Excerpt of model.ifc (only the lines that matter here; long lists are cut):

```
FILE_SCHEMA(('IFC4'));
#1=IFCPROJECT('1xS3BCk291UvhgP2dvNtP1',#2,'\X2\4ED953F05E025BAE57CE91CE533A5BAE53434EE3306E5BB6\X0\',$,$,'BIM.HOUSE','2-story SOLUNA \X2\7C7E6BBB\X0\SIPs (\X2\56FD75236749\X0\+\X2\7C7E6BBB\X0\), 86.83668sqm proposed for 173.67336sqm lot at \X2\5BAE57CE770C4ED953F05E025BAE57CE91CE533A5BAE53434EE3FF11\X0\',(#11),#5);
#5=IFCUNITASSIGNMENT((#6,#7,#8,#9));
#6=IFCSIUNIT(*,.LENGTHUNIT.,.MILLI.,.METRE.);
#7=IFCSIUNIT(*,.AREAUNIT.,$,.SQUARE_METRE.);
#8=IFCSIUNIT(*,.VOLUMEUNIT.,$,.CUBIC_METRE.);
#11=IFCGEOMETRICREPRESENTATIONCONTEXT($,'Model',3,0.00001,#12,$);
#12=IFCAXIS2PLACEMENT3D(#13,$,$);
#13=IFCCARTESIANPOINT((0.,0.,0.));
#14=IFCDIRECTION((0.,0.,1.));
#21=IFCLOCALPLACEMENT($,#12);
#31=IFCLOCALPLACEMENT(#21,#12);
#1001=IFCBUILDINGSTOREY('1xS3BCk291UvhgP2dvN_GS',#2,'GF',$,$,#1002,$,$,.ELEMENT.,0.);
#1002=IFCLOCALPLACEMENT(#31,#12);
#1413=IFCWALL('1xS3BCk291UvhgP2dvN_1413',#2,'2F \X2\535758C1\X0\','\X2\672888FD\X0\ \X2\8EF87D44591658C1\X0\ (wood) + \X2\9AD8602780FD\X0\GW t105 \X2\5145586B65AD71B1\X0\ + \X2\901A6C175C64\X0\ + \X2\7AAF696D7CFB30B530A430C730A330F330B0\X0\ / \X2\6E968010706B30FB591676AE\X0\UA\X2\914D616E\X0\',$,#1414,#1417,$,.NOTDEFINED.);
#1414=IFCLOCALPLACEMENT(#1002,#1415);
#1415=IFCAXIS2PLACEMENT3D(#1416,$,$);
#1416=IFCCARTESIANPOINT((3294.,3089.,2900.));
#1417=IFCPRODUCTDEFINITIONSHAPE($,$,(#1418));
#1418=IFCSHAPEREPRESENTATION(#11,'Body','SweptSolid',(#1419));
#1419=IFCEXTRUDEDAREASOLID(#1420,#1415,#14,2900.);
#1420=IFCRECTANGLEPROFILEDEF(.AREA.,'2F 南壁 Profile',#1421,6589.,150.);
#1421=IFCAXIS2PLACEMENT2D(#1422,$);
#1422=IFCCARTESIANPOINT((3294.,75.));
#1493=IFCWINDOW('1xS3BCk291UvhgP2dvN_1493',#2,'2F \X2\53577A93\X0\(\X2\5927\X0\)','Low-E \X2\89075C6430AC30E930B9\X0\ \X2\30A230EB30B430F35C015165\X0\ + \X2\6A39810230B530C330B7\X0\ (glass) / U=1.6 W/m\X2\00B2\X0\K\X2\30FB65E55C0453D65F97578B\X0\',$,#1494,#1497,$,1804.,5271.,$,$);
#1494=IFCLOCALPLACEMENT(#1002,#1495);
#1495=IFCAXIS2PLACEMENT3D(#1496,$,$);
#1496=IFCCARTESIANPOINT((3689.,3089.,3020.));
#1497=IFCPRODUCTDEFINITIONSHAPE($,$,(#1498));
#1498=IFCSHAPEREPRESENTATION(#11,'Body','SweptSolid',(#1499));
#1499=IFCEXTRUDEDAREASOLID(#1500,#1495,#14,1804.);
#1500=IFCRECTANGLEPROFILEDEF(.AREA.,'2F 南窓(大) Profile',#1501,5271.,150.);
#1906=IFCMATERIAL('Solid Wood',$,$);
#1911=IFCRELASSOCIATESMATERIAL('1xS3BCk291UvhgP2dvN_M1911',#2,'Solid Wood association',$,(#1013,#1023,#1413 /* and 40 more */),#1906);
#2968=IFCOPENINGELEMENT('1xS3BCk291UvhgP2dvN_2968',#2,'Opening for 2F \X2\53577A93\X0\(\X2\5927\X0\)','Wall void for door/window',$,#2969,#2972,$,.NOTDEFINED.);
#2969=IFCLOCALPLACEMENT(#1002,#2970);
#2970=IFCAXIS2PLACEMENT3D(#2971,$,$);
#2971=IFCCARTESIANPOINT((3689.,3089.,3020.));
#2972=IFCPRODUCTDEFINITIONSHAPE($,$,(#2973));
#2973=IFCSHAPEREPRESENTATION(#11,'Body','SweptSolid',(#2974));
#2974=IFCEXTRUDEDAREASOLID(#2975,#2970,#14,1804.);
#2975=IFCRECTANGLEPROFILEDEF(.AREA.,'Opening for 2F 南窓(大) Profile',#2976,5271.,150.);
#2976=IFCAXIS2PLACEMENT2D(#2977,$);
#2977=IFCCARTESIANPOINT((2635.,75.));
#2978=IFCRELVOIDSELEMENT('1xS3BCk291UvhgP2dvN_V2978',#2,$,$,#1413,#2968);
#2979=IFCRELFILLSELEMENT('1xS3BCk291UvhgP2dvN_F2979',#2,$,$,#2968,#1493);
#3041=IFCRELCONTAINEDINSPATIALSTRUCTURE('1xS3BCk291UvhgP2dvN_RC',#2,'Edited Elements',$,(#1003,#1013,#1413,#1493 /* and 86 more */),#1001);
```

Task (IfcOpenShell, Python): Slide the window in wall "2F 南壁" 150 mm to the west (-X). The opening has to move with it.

```python
import ifcopenshell
import ifcopenshell.api.geometry
import ifcopenshell.util.placement

model = ifcopenshell.open("model.ifc")

window = model.by_guid("1xS3BCk291UvhgP2dvN_1493")
opening = window.FillsVoids[0].RelatingOpeningElement
wall = opening.VoidsElements[0].RelatingBuildingElement

wall_matrix = ifcopenshell.util.placement.get_local_placement(wall.ObjectPlacement)
shift = wall_matrix[:3, 0] * -150.0
before = ifcopenshell.util.placement.get_local_placement(window.ObjectPlacement)[:3, 3].copy()

# The window is not placed relative to its opening, so move both.
for product in (opening, window):
    matrix = ifcopenshell.util.placement.get_local_placement(product.ObjectPlacement)
    matrix[:3, 3] += shift
    ifcopenshell.api.geometry.edit_object_placement(model, product=product, matrix=matrix, is_si=False)

after = ifcopenshell.util.placement.get_local_placement(window.ObjectPlacement)[:3, 3]
print("window moved by", (after - before).round(3) + 0.0)

model.write("model_rev.ifc")
```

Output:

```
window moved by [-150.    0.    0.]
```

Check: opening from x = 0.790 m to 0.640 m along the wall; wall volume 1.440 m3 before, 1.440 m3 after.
